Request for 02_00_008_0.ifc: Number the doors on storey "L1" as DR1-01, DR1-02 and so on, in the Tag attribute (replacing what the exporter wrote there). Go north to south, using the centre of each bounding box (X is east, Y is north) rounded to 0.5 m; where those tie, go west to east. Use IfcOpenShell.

First a look at what the model holds.

```python
import ifcopenshell
import ifcopenshell.util.element
import ifcopenshell.util.placement

model = ifcopenshell.open("02_00_008_0.ifc")
print(model.schema)
storey = next(s for s in model.by_type("IfcBuildingStorey") if s.Name == "L1")
doors = [e for e in ifcopenshell.util.element.get_decomposition(storey) if e.is_a("IfcDoor")]
for e in sorted(doors, key=lambda e: e.id()):
    origin = ifcopenshell.util.placement.get_local_placement(e.ObjectPlacement)[:3, 3]
    print(e.id(), e.Tag, e.Name, origin.round(2) + 0.0, sep=" | ")
```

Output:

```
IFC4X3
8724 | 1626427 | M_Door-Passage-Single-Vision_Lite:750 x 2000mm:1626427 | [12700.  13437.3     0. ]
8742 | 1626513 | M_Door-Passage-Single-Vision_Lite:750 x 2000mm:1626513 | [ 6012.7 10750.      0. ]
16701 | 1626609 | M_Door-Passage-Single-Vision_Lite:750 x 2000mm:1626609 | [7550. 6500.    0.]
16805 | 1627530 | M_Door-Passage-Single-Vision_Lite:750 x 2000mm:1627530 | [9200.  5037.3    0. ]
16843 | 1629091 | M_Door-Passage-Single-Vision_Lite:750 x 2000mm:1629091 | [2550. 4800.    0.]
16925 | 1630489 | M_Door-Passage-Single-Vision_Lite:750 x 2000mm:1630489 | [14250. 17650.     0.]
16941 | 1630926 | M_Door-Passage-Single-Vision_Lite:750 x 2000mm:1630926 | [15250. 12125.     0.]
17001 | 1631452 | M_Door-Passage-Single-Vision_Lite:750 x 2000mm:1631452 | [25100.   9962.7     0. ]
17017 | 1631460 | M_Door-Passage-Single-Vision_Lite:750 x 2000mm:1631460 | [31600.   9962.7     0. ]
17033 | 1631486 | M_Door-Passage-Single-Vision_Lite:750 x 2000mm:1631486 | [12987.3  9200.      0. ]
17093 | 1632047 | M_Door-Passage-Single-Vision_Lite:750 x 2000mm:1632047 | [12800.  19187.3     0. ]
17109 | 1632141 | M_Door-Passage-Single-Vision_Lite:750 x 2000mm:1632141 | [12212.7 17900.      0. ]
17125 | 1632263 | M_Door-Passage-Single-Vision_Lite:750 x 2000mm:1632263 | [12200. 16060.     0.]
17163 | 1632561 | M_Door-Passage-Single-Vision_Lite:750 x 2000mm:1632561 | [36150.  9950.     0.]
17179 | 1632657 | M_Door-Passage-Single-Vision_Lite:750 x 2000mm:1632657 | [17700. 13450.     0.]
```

```python
import ifcopenshell
import ifcopenshell.geom
import ifcopenshell.util.element
import ifcopenshell.util.shape

model = ifcopenshell.open("02_00_008_0.ifc")
settings = ifcopenshell.geom.settings()
settings.set("use-world-coords", True)


def centre(element):
    shape = ifcopenshell.geom.create_shape(settings, element)
    return ifcopenshell.util.shape.get_bbox_centroid(shape.geometry)


storey = next(s for s in model.by_type("IfcBuildingStorey") if s.Name == "L1")
doors = [e for e in ifcopenshell.util.element.get_decomposition(storey) if e.is_a("IfcDoor")]

# Insertion points can sit at a corner or the storey origin, so sort by the geometry (in metres).
centres = {e: centre(e) for e in doors}
doors.sort(key=lambda e: (-round(centres[e][1] / 0.5), centres[e][0]))

for i, e in enumerate(doors, start=1):
    number = f"DR1-{i:02d}"
    e.Tag = number
    print(e.id(), number)

model.write("02_00_008_0_rev.ifc")
```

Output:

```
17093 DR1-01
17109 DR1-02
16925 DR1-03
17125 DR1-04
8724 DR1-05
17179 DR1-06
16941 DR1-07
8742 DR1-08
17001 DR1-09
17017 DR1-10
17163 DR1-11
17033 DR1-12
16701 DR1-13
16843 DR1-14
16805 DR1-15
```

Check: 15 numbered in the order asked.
